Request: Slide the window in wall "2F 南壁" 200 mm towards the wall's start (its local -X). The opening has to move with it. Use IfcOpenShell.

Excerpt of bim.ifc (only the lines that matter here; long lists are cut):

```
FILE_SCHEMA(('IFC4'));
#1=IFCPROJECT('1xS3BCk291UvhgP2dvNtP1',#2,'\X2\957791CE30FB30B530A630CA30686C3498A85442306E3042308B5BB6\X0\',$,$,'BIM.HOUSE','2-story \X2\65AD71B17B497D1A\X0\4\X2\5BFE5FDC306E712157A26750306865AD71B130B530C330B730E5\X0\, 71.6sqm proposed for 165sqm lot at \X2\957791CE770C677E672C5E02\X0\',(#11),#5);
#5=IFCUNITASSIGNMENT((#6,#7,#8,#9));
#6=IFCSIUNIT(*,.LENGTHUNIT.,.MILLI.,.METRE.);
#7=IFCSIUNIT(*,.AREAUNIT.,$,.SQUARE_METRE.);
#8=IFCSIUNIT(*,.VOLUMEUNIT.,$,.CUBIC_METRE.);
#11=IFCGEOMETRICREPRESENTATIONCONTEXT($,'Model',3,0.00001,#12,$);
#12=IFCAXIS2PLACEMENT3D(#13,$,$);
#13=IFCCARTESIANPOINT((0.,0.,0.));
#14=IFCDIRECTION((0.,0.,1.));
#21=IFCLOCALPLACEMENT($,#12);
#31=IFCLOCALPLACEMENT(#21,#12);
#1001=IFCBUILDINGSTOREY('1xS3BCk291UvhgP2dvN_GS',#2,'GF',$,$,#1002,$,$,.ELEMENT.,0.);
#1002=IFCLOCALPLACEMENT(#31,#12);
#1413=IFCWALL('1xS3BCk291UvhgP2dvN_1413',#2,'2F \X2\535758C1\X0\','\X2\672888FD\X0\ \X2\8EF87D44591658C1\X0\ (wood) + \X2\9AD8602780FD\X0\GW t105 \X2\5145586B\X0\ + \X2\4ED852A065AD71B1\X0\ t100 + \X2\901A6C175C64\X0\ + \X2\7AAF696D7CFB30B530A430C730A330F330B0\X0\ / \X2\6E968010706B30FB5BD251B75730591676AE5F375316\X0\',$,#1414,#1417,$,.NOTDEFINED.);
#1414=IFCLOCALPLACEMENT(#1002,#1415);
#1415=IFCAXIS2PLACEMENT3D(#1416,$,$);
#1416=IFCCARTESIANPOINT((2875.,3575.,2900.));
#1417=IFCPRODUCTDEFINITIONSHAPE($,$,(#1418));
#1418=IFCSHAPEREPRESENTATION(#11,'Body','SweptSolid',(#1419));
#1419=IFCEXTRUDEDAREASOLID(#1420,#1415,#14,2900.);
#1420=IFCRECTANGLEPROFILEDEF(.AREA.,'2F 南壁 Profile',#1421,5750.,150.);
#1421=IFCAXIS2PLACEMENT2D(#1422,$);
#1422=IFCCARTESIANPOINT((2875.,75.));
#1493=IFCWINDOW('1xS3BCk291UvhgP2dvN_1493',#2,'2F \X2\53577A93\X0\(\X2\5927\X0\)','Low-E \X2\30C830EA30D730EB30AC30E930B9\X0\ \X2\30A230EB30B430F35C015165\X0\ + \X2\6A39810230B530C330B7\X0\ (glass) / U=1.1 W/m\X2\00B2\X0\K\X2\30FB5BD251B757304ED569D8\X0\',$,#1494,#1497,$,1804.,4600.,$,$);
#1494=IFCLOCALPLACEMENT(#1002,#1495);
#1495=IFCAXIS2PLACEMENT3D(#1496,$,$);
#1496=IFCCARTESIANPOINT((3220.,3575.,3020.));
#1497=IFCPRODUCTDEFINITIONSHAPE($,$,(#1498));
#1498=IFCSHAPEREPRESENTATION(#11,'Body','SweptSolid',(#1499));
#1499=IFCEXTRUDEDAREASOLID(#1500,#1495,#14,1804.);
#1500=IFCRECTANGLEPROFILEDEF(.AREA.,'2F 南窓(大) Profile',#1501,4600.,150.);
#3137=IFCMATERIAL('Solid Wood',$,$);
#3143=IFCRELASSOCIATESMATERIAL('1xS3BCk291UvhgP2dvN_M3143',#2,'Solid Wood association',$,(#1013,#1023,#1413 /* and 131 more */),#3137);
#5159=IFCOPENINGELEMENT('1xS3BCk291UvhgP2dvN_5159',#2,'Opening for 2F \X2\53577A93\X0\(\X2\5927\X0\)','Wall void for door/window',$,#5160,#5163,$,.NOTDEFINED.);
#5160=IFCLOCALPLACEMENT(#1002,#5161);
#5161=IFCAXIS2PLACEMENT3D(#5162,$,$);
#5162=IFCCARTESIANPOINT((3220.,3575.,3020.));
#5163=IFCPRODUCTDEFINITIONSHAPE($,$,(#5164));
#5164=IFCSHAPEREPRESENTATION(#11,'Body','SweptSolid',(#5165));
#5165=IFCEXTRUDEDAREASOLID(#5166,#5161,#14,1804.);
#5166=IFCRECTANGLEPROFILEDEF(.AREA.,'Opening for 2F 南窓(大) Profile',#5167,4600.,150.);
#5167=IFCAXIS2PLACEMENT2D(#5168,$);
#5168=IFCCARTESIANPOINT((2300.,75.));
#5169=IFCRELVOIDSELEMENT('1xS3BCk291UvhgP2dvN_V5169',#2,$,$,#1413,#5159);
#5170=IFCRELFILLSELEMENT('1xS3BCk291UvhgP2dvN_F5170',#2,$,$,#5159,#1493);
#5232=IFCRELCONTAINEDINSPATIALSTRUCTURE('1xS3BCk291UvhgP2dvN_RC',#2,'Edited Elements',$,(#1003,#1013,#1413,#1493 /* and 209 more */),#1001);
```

```python
import ifcopenshell
import ifcopenshell.api.geometry
import ifcopenshell.util.placement
import ifcopenshell.util.unit

model = ifcopenshell.open("bim.ifc")
unit_scale = ifcopenshell.util.unit.calculate_unit_scale(model)

window = model.by_guid("1xS3BCk291UvhgP2dvN_1493")
opening = window.FillsVoids[0].RelatingOpeningElement
wall = opening.VoidsElements[0].RelatingBuildingElement

wall_matrix = ifcopenshell.util.placement.get_local_placement(wall.ObjectPlacement)
shift = wall_matrix[:3, 0] * -0.2 / unit_scale
before = ifcopenshell.util.placement.get_local_placement(window.ObjectPlacement)[:3, 3].copy()

# The window is not placed relative to its opening, so move both.
for product in (opening, window):
    matrix = ifcopenshell.util.placement.get_local_placement(product.ObjectPlacement)
    matrix[:3, 3] += shift
    ifcopenshell.api.geometry.edit_object_placement(model, product=product, matrix=matrix, is_si=False)

after = ifcopenshell.util.placement.get_local_placement(window.ObjectPlacement)[:3, 3]
print("window moved by", (after - before).round(3) + 0.0)

model.write("bim_rev.ifc")
```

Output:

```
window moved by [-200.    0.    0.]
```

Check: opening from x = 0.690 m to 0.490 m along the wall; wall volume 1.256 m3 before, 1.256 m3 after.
